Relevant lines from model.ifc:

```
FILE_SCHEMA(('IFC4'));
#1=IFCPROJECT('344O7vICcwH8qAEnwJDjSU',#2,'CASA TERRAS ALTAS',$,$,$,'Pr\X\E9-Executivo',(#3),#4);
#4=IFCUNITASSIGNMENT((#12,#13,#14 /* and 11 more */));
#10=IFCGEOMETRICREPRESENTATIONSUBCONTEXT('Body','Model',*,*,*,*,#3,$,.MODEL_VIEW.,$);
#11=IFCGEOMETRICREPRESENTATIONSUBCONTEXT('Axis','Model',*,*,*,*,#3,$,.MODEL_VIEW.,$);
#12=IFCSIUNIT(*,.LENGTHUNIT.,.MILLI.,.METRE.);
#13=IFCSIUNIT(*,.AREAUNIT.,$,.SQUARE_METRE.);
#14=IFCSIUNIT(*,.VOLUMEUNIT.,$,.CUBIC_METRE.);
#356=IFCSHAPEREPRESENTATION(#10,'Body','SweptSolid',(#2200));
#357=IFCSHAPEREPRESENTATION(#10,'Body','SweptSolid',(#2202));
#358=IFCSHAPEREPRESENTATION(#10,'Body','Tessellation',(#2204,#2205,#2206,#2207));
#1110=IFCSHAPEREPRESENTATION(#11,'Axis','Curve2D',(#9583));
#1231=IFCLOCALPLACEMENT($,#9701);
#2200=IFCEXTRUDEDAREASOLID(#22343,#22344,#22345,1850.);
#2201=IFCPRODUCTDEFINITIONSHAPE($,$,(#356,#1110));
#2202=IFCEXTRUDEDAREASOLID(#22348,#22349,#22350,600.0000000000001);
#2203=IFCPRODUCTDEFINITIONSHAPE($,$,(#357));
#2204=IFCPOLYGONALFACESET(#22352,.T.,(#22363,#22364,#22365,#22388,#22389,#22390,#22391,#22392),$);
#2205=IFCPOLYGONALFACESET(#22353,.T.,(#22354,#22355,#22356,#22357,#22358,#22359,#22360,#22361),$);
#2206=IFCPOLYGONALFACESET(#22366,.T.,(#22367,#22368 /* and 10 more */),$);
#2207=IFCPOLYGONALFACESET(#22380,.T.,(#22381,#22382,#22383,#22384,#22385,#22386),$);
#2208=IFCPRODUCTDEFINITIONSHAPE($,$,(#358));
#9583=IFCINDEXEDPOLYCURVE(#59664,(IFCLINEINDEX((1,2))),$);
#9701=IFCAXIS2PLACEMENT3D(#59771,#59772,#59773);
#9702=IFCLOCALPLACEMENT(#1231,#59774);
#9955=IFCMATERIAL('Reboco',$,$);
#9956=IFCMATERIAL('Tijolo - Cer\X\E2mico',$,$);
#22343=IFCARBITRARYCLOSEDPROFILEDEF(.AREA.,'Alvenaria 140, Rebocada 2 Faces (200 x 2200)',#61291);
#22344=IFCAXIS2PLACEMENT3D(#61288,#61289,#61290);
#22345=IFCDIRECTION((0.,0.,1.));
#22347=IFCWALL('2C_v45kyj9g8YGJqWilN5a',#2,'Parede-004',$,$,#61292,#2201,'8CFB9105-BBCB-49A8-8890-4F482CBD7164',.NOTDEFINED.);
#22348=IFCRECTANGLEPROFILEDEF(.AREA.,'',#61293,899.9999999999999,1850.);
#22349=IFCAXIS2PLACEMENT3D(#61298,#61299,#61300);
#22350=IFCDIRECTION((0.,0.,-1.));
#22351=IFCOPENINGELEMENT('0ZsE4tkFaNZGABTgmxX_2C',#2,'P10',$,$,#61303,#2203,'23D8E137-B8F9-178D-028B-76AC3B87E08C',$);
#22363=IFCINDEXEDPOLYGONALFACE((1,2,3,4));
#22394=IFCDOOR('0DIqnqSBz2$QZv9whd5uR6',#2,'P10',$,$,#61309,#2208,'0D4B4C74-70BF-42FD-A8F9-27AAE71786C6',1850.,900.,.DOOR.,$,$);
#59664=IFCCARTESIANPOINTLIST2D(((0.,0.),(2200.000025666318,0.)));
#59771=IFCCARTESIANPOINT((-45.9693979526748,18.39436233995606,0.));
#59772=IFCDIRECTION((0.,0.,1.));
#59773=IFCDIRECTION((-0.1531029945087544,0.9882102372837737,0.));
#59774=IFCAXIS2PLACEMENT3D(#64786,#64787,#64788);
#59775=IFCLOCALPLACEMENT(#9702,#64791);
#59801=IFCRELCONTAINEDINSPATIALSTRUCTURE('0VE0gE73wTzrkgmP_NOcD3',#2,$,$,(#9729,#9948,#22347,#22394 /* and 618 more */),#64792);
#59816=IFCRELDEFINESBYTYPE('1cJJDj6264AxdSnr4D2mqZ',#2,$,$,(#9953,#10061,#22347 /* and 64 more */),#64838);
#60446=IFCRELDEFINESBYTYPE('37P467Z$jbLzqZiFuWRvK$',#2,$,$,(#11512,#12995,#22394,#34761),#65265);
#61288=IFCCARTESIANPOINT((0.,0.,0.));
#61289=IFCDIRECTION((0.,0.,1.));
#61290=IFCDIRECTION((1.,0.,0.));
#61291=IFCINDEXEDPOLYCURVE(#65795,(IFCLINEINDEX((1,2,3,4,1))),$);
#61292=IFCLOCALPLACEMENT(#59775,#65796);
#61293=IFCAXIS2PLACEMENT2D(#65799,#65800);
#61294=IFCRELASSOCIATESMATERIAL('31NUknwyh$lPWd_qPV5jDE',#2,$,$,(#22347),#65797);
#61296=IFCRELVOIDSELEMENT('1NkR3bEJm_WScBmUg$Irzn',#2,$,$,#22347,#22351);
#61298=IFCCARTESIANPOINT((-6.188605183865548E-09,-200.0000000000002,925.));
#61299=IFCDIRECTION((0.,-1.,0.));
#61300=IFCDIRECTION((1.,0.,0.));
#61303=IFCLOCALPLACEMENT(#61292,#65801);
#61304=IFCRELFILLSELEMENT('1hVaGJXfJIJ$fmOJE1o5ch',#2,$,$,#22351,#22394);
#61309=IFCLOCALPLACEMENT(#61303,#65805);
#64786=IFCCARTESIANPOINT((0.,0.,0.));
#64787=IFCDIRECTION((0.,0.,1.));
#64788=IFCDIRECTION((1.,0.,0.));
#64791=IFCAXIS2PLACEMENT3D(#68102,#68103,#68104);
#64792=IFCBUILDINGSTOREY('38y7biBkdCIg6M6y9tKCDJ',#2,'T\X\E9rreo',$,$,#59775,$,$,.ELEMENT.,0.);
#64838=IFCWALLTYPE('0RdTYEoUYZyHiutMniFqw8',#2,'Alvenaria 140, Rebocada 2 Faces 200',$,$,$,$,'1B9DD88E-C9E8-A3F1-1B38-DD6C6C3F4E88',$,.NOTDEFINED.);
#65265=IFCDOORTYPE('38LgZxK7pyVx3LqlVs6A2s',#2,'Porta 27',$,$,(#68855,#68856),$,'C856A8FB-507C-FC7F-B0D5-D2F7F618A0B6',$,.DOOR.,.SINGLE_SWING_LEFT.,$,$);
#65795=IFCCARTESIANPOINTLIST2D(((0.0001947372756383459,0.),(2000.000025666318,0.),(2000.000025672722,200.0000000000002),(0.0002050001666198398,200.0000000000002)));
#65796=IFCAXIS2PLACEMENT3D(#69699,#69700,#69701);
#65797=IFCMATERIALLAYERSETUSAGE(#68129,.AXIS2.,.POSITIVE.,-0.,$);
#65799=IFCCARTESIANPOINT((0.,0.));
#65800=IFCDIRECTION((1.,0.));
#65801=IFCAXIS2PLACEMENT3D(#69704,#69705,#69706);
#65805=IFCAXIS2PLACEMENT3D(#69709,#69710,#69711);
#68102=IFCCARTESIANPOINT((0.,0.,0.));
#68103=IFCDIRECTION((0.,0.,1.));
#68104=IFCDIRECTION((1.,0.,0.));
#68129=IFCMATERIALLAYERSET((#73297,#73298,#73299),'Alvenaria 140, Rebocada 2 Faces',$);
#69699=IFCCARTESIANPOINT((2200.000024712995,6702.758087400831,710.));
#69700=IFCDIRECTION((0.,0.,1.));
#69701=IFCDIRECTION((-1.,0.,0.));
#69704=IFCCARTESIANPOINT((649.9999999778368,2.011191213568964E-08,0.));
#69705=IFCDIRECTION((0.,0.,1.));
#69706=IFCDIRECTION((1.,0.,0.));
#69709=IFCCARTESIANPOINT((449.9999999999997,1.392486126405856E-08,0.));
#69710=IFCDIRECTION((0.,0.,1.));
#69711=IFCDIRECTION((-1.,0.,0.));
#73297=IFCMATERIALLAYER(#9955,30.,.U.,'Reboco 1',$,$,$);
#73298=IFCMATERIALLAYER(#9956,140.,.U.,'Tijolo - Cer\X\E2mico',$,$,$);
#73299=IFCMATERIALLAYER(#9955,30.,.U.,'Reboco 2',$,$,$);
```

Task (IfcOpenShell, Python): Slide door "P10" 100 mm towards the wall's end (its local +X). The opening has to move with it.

```python
import ifcopenshell
import ifcopenshell.api.geometry
import ifcopenshell.util.placement

model = ifcopenshell.open("model.ifc")

door = model.by_guid("0DIqnqSBz2$QZv9whd5uR6")
opening = door.FillsVoids[0].RelatingOpeningElement
wall = opening.VoidsElements[0].RelatingBuildingElement

wall_matrix = ifcopenshell.util.placement.get_local_placement(wall.ObjectPlacement)
shift = wall_matrix[:3, 0] * 100.0
before = ifcopenshell.util.placement.get_local_placement(door.ObjectPlacement)[:3, 3].copy()

# The door is placed relative to its opening, so it follows when the opening moves.
matrix = ifcopenshell.util.placement.get_local_placement(opening.ObjectPlacement)
matrix[:3, 3] += shift
ifcopenshell.api.geometry.edit_object_placement(
    model, product=opening, matrix=matrix, is_si=False, should_transform_children=True
)

after = ifcopenshell.util.placement.get_local_placement(door.ObjectPlacement)[:3, 3]
print("door moved by", (after - before).round(3) + 0.0)

model.write("model_v2.ifc")
```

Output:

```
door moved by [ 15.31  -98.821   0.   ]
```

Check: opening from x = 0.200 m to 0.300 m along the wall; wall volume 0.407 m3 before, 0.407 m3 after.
